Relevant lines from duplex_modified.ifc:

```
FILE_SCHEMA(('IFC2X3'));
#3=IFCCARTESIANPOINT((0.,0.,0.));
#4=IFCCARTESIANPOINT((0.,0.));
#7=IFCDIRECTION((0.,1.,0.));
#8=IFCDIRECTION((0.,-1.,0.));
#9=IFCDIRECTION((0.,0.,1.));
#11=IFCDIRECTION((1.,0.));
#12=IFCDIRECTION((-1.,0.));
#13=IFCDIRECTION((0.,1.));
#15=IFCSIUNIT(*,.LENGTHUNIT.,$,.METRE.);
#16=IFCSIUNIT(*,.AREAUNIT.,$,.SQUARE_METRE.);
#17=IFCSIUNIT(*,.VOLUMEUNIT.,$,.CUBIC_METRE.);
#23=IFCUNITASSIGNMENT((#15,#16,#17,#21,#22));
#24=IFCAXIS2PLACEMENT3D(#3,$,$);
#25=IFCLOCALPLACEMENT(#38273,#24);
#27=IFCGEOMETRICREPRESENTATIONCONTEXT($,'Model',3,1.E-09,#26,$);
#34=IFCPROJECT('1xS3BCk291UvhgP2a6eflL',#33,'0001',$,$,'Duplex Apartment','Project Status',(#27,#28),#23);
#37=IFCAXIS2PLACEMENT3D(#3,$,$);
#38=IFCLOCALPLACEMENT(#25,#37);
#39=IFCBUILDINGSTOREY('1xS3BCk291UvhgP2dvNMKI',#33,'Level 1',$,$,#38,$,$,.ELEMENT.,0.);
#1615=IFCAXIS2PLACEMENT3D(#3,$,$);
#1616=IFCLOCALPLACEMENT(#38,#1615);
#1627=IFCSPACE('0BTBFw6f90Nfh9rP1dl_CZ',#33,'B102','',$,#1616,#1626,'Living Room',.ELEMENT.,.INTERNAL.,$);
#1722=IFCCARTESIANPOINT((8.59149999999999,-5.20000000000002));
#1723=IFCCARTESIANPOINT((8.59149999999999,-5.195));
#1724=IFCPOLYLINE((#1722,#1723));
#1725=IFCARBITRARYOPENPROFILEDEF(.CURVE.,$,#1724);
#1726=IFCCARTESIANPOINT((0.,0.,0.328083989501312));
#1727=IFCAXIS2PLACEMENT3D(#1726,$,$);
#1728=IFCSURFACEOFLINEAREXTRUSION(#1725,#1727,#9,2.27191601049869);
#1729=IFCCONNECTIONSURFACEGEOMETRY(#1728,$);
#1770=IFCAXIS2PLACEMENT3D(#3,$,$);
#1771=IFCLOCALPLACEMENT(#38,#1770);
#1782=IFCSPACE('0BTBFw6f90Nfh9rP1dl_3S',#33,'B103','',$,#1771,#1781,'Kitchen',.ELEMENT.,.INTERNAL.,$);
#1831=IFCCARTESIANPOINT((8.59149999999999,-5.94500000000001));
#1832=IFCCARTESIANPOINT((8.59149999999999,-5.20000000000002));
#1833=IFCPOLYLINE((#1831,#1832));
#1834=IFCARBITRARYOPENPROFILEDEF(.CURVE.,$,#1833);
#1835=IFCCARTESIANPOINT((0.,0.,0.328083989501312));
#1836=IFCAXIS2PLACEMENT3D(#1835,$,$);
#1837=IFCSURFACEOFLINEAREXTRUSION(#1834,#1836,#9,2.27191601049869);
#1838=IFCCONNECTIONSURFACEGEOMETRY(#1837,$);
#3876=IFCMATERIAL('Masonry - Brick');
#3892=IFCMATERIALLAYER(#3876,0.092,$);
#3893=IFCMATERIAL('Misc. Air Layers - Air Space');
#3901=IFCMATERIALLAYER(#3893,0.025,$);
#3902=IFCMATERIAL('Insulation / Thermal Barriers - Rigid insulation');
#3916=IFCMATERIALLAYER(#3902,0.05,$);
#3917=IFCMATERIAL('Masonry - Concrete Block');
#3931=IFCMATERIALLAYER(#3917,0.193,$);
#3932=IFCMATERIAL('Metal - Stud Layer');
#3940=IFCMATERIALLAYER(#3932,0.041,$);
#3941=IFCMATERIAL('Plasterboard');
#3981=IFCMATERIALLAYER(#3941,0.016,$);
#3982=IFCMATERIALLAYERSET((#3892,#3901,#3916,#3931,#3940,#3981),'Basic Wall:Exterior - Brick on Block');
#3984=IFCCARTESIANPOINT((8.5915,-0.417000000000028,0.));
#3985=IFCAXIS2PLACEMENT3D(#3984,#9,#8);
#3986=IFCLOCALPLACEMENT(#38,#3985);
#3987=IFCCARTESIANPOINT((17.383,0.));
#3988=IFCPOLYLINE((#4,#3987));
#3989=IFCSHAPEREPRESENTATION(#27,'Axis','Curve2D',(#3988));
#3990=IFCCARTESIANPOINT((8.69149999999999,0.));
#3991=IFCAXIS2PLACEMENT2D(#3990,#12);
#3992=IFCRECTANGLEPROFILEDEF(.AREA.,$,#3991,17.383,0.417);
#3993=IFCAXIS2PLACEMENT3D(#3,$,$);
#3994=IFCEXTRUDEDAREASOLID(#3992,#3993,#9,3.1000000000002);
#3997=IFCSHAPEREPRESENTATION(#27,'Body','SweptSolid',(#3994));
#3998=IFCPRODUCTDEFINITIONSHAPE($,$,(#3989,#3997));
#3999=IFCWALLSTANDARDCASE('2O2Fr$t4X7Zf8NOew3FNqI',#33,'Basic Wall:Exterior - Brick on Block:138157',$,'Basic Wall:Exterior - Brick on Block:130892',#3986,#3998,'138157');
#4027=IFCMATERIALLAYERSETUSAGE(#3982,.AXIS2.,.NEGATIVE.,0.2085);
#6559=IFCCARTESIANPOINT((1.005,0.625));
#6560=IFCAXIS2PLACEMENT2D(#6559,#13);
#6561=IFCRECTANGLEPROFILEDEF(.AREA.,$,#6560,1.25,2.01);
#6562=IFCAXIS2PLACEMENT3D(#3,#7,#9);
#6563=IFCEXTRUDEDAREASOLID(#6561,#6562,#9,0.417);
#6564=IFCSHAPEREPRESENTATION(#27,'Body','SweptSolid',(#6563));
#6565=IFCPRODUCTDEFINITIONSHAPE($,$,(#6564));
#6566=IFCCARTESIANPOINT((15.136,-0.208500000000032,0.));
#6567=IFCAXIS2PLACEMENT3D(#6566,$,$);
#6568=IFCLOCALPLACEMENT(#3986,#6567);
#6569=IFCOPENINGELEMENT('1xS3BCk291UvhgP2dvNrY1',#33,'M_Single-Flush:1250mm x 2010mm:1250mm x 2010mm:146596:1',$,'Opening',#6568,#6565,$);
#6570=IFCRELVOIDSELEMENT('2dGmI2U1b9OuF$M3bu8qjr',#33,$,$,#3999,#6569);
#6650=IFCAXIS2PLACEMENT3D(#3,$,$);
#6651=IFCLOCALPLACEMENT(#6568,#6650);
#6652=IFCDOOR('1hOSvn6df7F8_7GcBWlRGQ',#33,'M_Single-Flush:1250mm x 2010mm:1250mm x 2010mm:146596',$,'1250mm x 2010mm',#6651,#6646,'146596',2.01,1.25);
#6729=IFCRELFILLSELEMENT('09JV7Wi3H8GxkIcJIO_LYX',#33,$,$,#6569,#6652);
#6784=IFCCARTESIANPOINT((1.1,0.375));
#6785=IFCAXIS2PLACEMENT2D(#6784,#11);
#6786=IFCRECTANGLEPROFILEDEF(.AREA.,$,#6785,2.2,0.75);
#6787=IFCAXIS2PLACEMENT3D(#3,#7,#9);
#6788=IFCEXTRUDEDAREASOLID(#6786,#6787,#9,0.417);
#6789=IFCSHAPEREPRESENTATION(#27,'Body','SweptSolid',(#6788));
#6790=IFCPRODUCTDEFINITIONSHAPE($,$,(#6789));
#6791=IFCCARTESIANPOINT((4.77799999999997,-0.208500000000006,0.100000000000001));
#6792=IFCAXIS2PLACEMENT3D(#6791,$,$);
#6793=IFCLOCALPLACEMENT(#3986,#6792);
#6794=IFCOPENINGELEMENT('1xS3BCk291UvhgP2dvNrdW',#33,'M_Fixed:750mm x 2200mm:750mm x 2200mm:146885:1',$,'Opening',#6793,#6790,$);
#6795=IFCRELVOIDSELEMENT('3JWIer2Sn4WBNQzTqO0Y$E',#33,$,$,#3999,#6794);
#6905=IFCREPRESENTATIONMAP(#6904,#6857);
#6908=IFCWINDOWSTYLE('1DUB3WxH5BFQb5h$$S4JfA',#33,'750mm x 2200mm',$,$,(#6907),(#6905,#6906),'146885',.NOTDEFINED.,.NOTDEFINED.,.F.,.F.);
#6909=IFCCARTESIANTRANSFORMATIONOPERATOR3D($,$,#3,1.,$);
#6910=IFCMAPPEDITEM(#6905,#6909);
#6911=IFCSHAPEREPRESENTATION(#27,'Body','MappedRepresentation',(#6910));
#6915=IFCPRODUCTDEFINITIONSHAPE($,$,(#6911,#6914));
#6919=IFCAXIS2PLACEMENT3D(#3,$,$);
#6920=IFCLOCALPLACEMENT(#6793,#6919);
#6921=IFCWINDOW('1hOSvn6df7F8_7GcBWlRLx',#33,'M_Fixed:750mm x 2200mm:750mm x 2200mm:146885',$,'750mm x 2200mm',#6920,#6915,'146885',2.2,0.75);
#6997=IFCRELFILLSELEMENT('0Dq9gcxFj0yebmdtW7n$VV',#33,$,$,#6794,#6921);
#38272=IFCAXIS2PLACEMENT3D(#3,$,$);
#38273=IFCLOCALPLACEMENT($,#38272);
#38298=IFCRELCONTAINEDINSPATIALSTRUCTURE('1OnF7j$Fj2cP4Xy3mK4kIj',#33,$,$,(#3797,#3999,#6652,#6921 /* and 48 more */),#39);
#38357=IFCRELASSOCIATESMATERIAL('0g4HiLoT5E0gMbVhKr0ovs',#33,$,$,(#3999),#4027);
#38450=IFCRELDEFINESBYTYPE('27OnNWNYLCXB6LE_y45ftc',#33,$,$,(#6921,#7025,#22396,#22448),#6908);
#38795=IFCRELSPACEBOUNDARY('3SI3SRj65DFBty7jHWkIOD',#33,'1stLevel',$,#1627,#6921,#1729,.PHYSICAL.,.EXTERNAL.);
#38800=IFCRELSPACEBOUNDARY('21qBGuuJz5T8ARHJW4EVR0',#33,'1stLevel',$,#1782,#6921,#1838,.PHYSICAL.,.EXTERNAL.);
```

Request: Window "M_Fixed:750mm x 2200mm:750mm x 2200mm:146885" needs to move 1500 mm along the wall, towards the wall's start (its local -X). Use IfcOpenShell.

```python
import numpy as np
import ifcopenshell
import ifcopenshell.api.geometry
import ifcopenshell.util.placement
import ifcopenshell.util.unit

model = ifcopenshell.open("duplex_modified.ifc")
unit_scale = ifcopenshell.util.unit.calculate_unit_scale(model)

window = model.by_guid("1hOSvn6df7F8_7GcBWlRLx")
opening = window.FillsVoids[0].RelatingOpeningElement
wall = opening.VoidsElements[0].RelatingBuildingElement

wall_matrix = ifcopenshell.util.placement.get_local_placement(wall.ObjectPlacement)
shift = wall_matrix[:3, 0] * -1.5 / unit_scale
before = ifcopenshell.util.placement.get_local_placement(window.ObjectPlacement)[:3, 3].copy()

# The window is placed relative to its opening, so it follows when the opening moves.
matrix = ifcopenshell.util.placement.get_local_placement(opening.ObjectPlacement)
matrix[:3, 3] += shift
ifcopenshell.api.geometry.edit_object_placement(
    model, product=opening, matrix=matrix, is_si=False, should_transform_children=True
)

# Space boundary surfaces are stored in each space's coordinates; move them too.
for rel in window.ProvidesBoundaries:
    if not rel.ConnectionGeometry:
        continue
    surface = rel.ConnectionGeometry.SurfaceOnRelatingElement
    space_matrix = ifcopenshell.util.placement.get_local_placement(rel.RelatingSpace.ObjectPlacement)
    point = np.array(surface.Position.Location.Coordinates) + space_matrix[:3, :3].T @ shift
    surface.Position = model.createIfcAxis2Placement3D(
        model.createIfcCartesianPoint(point.tolist()), surface.Position.Axis, surface.Position.RefDirection
    )

after = ifcopenshell.util.placement.get_local_placement(window.ObjectPlacement)[:3, 3]
print("window moved by", (after - before).round(3) + 0.0)

model.write("duplex_modified_updated.ifc")
```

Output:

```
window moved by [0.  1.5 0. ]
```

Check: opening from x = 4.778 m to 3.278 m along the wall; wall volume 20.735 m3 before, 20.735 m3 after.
